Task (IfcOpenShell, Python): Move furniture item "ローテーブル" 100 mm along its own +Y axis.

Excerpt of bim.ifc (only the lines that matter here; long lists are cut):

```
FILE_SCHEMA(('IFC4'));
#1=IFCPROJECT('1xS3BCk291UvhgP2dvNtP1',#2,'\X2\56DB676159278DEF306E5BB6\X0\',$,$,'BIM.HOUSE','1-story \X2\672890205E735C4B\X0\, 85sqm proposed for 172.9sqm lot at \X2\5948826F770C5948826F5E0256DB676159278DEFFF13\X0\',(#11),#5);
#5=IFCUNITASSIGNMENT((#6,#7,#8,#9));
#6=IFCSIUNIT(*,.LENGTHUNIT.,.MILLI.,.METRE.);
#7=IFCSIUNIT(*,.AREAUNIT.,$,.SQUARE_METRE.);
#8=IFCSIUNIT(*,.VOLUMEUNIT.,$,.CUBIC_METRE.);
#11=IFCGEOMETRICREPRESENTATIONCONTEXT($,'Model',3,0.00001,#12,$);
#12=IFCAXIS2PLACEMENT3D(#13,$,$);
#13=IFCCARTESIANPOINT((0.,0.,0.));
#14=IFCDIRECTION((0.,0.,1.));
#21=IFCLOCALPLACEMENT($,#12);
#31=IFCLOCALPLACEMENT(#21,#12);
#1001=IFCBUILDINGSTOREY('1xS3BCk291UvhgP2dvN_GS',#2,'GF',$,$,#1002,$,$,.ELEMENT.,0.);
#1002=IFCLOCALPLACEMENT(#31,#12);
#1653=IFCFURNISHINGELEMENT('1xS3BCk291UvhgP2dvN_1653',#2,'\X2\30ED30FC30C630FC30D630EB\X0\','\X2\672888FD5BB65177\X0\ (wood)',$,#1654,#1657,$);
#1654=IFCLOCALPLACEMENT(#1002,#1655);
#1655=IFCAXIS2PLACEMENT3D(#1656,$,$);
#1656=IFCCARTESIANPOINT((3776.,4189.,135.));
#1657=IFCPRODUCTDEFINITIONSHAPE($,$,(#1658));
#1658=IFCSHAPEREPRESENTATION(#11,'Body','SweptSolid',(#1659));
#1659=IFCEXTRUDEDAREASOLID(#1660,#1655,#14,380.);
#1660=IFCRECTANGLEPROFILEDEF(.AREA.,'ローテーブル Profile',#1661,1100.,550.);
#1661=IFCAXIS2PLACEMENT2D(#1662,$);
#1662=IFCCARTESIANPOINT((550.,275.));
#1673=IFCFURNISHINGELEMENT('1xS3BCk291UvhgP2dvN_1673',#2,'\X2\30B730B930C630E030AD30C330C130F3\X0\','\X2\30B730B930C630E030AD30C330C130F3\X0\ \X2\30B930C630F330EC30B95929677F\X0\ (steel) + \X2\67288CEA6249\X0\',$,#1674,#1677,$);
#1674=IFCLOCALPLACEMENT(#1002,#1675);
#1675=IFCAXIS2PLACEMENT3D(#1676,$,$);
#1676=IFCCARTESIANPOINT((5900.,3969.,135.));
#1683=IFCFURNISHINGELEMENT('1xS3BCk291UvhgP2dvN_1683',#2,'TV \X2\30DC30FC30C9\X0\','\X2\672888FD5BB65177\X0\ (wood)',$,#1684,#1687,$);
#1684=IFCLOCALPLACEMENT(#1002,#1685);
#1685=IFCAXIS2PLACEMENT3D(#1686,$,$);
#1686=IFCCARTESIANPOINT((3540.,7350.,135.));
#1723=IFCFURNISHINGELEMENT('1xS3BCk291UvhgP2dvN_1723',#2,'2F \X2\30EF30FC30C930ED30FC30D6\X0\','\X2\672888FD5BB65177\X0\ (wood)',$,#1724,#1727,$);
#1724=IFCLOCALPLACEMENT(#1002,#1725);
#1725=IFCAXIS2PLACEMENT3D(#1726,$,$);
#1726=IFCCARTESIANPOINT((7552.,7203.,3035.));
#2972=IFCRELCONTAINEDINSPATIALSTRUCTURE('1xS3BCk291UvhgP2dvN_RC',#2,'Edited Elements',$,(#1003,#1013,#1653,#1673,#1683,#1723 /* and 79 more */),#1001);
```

```python
import ifcopenshell
import ifcopenshell.api.geometry
import ifcopenshell.util.placement
import ifcopenshell.util.unit

model = ifcopenshell.open("bim.ifc")
unit_scale = ifcopenshell.util.unit.calculate_unit_scale(model)

item = model.by_guid("1xS3BCk291UvhgP2dvN_1653")
matrix = ifcopenshell.util.placement.get_local_placement(item.ObjectPlacement)
matrix[:3, 3] += matrix[:3, 1] * 0.1 / unit_scale
ifcopenshell.api.geometry.edit_object_placement(model, product=item, matrix=matrix, is_si=False)

print(ifcopenshell.util.placement.get_local_placement(item.ObjectPlacement).round(3) + 0.0)

model.write("bim_updated.ifc")
```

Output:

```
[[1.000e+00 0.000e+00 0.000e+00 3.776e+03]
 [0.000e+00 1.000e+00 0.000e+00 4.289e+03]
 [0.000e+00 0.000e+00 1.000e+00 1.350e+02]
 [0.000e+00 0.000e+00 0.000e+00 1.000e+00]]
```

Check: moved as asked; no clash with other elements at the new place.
